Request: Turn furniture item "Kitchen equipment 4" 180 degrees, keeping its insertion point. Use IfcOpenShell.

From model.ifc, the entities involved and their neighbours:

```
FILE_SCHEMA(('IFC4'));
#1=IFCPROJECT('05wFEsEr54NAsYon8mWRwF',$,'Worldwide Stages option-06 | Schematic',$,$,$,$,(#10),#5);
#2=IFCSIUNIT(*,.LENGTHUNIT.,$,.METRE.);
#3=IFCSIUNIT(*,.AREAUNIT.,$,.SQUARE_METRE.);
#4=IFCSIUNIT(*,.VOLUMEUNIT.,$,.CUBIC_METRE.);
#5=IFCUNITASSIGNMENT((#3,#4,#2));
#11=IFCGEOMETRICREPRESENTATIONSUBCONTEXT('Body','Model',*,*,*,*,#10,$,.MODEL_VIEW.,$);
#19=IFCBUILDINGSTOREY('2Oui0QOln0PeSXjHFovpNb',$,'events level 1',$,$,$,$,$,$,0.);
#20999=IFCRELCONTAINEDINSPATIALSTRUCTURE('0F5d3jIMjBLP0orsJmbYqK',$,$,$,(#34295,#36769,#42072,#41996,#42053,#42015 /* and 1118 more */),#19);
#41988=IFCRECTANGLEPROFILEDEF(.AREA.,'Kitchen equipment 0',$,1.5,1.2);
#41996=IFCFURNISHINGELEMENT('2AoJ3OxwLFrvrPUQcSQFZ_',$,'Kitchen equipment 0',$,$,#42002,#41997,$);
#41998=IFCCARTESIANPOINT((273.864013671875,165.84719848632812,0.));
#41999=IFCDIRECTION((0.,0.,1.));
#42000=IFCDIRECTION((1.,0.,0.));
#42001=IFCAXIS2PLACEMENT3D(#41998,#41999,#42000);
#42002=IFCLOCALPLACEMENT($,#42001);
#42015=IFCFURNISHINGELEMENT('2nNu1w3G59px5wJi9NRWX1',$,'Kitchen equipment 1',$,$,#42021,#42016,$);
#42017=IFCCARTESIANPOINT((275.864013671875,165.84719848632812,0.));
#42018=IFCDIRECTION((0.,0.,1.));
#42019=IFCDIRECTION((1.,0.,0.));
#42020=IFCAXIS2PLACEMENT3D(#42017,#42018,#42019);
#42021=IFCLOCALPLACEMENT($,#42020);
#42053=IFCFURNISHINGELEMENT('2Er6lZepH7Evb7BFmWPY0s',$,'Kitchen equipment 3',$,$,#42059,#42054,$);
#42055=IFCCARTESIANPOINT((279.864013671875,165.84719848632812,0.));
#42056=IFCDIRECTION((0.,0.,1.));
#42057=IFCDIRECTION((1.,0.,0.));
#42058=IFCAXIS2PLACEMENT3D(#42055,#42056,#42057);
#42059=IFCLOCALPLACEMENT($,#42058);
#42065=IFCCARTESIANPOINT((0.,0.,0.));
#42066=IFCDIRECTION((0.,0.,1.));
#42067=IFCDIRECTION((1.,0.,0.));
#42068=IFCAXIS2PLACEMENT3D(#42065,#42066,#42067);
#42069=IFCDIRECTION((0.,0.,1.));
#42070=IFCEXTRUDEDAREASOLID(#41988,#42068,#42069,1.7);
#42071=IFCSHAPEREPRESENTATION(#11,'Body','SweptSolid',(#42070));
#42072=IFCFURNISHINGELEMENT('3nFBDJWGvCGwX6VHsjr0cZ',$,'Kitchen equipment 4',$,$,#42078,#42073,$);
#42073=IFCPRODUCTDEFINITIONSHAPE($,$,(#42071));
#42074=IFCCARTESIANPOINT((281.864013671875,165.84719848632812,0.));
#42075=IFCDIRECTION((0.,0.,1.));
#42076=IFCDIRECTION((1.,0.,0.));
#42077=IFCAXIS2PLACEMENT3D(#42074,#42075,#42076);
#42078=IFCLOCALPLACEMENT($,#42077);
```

```python
import ifcopenshell
import ifcopenshell.api.geometry
import ifcopenshell.util.placement

model = ifcopenshell.open("model.ifc")

item = model.by_guid("3nFBDJWGvCGwX6VHsjr0cZ")
matrix = ifcopenshell.util.placement.get_local_placement(item.ObjectPlacement)
matrix = matrix @ ifcopenshell.util.placement.rotation(180, "Z")
ifcopenshell.api.geometry.edit_object_placement(model, product=item, matrix=matrix, is_si=False)

print(ifcopenshell.util.placement.get_local_placement(item.ObjectPlacement).round(3) + 0.0)

model.write("model-out.ifc")
```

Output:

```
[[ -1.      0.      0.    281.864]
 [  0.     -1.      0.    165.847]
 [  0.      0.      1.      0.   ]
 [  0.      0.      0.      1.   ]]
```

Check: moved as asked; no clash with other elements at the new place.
